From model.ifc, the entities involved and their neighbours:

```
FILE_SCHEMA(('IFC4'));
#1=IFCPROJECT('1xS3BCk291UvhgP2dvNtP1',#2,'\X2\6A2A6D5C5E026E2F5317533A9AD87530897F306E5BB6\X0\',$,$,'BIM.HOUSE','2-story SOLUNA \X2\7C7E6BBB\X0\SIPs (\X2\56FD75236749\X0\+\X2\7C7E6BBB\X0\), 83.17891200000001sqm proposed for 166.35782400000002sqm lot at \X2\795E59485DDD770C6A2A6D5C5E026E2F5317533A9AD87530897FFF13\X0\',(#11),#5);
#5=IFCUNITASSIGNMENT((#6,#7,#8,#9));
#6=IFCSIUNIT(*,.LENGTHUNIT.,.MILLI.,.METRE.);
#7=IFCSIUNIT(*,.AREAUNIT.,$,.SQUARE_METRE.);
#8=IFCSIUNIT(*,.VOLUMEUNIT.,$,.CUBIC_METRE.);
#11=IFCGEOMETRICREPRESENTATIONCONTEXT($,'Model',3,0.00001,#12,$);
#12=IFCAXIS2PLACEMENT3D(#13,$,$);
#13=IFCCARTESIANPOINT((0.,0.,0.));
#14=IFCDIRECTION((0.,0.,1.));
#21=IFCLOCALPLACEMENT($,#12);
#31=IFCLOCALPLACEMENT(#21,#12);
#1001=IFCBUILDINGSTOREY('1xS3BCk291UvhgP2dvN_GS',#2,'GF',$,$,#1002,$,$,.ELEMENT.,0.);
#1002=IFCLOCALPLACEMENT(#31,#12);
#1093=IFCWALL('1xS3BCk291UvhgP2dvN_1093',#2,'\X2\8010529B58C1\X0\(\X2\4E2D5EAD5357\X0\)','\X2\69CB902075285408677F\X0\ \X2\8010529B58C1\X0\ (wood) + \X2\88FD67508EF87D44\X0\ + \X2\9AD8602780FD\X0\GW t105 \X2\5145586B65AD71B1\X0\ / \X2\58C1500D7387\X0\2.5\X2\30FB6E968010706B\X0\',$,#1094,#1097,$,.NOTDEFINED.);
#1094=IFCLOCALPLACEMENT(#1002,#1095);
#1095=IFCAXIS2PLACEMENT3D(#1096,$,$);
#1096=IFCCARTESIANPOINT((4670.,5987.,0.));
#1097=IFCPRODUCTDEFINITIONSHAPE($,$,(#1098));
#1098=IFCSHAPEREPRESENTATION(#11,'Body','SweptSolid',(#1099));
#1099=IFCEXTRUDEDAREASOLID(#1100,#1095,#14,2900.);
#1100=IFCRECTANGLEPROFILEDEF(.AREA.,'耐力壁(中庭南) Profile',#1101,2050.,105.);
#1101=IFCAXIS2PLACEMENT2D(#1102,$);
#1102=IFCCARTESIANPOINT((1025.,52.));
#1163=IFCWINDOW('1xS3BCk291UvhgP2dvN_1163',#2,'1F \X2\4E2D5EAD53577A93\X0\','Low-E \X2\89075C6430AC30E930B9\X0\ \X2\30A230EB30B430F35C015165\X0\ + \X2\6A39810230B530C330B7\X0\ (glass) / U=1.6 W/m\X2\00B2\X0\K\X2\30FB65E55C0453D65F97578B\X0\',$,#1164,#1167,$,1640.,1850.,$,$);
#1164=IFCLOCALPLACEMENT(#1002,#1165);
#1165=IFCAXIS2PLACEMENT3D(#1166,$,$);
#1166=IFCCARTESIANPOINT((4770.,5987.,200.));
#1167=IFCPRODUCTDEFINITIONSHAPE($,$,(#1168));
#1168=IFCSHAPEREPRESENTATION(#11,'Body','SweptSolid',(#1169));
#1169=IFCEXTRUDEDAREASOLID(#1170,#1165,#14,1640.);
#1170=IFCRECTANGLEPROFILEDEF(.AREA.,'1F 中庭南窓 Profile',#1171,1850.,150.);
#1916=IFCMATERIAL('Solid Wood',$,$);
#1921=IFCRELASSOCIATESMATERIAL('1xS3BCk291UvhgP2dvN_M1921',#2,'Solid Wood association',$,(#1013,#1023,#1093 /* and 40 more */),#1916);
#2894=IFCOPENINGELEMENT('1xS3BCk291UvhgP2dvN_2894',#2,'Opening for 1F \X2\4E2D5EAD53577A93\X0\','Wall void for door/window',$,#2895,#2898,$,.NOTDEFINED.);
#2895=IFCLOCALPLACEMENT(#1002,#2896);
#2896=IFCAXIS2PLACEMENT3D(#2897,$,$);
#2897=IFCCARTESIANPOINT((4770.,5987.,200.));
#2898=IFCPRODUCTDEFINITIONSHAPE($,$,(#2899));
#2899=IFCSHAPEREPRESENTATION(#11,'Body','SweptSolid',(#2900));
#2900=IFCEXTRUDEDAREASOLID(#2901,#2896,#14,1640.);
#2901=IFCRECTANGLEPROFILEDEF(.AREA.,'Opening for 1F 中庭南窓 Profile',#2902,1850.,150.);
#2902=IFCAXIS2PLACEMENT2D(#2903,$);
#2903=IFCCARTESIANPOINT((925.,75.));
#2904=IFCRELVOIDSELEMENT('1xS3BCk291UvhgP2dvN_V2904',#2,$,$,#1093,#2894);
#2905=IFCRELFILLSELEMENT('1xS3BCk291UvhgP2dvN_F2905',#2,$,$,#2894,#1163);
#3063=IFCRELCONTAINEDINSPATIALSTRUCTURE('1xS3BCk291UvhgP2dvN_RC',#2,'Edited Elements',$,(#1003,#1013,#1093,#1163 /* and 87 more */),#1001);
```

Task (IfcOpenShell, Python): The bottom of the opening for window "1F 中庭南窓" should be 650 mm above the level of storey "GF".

```python
import numpy as np
import ifcopenshell
import ifcopenshell.api.geometry
import ifcopenshell.geom
import ifcopenshell.util.element
import ifcopenshell.util.placement
import ifcopenshell.util.shape
import ifcopenshell.util.unit

model = ifcopenshell.open("model.ifc")
unit_scale = ifcopenshell.util.unit.calculate_unit_scale(model)

window = model.by_id(1163)
opening = window.FillsVoids[0].RelatingOpeningElement
storey = ifcopenshell.util.element.get_container(window, ifc_class="IfcBuildingStorey")
level = ifcopenshell.util.placement.get_local_placement(storey.ObjectPlacement)[2, 3]

# The opening's origin need not be at the sill, so measure its lowest point.
shape = ifcopenshell.geom.create_shape(ifcopenshell.geom.settings(), opening)
bottom = ifcopenshell.util.shape.get_shape_bottom_elevation(shape, shape.geometry) / unit_scale
dz = level + 650.0 - bottom

shift = np.array([0.0, 0.0, dz])
# The window is not placed relative to its opening, so move both.
for product in (opening, window):
    matrix = ifcopenshell.util.placement.get_local_placement(product.ObjectPlacement)
    matrix[:3, 3] += shift
    ifcopenshell.api.geometry.edit_object_placement(model, product=product, matrix=matrix, is_si=False)

print(f"moved by {dz * unit_scale:+.3f} m")

model.write("model_v2.ifc")
```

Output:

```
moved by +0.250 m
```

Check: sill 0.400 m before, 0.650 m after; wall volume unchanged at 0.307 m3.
